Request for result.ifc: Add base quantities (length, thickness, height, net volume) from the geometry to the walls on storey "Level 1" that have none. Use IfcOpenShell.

First a look at what the model holds.

```python
import ifcopenshell
import ifcopenshell.util.element
import ifcopenshell.util.unit

model = ifcopenshell.open("result.ifc")
print(model.schema)
for unit_type in ("LENGTHUNIT", "AREAUNIT", "VOLUMEUNIT"):
    print(unit_type, ifcopenshell.util.unit.calculate_unit_scale(model, unit_type))
storey = next(s for s in model.by_type("IfcBuildingStorey") if s.Name == "Level 1")
walls = [e for e in ifcopenshell.util.element.get_decomposition(storey) if e.is_a("IfcWall")]
for e in sorted(walls, key=lambda e: e.id()):
    print(e.id(), e.is_a(), e.Name, list(ifcopenshell.util.element.get_psets(e, qtos_only=True)), sep=" | ")
```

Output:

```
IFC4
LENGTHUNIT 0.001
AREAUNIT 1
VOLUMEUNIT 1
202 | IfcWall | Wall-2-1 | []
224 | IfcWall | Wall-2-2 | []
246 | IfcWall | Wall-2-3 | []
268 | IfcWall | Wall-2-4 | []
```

```python
import ifcopenshell
import ifcopenshell.api.pset
import ifcopenshell.geom
import ifcopenshell.util.element
import ifcopenshell.util.shape
import ifcopenshell.util.unit

model = ifcopenshell.open("result.ifc")
unit_scale = ifcopenshell.util.unit.calculate_unit_scale(model)
volume_scale = ifcopenshell.util.unit.calculate_unit_scale(model, "VOLUMEUNIT")
settings = ifcopenshell.geom.settings()

storey = next(s for s in model.by_type("IfcBuildingStorey") if s.Name == "Level 1")
walls = [e for e in ifcopenshell.util.element.get_decomposition(storey) if e.is_a("IfcWall")]

for e in sorted(walls, key=lambda e: e.id()):
    if ifcopenshell.util.element.get_psets(e, qtos_only=True, should_inherit=False):
        continue
    # Geometry comes back in metres, in the element's own axes.
    shape = ifcopenshell.geom.create_shape(settings, e)
    values = {
        "Length": ifcopenshell.util.shape.get_x(shape.geometry) / unit_scale,
        "Width": ifcopenshell.util.shape.get_y(shape.geometry) / unit_scale,
        "Height": ifcopenshell.util.shape.get_z(shape.geometry) / unit_scale,
        "NetVolume": ifcopenshell.util.shape.get_volume(shape.geometry) / volume_scale,
    }
    qto = ifcopenshell.api.pset.add_qto(model, product=e, name="Qto_WallBaseQuantities")
    ifcopenshell.api.pset.edit_qto(model, qto=qto, properties=values)
    print(e.id(), {k: round(v, 3) for k, v in values.items()})

model.write("result_v2.ifc")
```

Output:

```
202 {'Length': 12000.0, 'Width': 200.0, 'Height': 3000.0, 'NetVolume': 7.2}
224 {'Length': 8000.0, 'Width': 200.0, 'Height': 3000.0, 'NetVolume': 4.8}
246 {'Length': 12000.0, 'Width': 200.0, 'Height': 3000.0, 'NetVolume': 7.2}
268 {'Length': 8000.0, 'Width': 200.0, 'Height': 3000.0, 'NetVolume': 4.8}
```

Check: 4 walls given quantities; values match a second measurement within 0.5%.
